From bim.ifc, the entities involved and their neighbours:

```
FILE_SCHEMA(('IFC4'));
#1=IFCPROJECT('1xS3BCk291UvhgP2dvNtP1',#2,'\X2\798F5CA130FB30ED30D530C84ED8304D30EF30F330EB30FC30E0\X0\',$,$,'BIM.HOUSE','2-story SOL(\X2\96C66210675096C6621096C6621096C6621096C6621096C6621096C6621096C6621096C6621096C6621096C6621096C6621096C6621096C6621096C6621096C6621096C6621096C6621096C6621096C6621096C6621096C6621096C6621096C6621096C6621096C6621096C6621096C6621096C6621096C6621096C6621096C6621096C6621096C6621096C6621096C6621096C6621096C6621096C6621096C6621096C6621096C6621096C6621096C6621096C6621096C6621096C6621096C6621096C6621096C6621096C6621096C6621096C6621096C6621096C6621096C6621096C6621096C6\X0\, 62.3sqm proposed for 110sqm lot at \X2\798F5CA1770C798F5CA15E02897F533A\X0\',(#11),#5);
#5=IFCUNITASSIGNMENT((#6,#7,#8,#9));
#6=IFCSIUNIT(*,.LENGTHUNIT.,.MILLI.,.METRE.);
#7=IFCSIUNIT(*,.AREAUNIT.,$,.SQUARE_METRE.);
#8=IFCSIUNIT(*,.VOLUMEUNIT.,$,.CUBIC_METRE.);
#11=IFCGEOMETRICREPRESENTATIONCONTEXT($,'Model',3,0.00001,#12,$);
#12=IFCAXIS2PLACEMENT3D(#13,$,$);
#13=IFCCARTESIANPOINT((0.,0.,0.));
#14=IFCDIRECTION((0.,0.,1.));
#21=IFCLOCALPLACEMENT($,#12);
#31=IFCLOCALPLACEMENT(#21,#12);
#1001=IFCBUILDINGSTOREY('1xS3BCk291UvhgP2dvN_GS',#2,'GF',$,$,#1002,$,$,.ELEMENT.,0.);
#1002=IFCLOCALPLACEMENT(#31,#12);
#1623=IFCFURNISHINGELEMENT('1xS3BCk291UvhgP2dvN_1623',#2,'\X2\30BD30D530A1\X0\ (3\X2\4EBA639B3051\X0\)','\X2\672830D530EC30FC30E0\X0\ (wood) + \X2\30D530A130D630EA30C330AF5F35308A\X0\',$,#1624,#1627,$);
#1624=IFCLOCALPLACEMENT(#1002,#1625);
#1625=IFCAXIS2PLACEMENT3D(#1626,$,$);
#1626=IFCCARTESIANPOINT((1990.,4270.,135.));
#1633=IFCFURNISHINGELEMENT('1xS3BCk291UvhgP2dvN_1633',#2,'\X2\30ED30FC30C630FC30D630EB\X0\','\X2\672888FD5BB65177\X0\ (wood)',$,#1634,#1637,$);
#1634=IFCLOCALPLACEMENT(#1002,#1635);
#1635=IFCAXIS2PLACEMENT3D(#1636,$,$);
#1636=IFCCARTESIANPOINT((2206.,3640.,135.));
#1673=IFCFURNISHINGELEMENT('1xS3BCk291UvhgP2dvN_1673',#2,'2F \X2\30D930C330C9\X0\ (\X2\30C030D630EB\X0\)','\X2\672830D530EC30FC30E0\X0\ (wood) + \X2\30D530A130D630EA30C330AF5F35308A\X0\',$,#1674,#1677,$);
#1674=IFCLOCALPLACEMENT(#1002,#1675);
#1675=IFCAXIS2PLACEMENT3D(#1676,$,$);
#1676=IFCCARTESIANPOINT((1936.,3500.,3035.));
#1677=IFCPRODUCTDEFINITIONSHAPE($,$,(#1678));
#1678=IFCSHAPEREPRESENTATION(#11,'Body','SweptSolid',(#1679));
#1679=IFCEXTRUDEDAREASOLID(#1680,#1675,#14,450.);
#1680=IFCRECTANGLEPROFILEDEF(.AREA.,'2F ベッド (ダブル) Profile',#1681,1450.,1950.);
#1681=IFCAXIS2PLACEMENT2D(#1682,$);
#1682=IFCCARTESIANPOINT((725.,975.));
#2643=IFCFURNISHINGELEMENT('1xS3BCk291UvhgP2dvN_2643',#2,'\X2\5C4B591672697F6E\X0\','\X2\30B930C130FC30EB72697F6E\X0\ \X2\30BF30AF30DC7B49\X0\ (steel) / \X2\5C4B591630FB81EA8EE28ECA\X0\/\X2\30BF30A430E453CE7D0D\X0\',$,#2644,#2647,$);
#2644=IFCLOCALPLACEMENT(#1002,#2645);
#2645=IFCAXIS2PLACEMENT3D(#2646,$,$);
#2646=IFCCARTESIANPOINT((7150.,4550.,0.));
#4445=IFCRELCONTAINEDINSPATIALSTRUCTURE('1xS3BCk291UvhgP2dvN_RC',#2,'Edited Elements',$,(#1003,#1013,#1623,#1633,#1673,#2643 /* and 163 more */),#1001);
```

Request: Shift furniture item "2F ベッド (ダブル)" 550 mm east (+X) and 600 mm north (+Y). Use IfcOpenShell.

```python
import ifcopenshell
import ifcopenshell.api.geometry
import ifcopenshell.util.placement
import ifcopenshell.util.unit

model = ifcopenshell.open("bim.ifc")
unit_scale = ifcopenshell.util.unit.calculate_unit_scale(model)

item = model.by_guid("1xS3BCk291UvhgP2dvN_1673")
matrix = ifcopenshell.util.placement.get_local_placement(item.ObjectPlacement)
matrix[0, 3] += 0.55 / unit_scale
matrix[1, 3] += 0.6 / unit_scale
ifcopenshell.api.geometry.edit_object_placement(model, product=item, matrix=matrix, is_si=False)

print(ifcopenshell.util.placement.get_local_placement(item.ObjectPlacement).round(3) + 0.0)

model.write("bim_updated.ifc")
```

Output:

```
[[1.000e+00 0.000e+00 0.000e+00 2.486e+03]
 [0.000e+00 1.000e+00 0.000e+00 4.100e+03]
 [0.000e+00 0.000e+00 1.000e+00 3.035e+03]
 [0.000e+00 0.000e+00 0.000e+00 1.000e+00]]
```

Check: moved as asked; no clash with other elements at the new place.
